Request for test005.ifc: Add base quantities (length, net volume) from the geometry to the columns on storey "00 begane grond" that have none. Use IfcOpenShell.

First a look at what the model holds.

```python
import ifcopenshell
import ifcopenshell.util.element
import ifcopenshell.util.unit

model = ifcopenshell.open("test005.ifc")
print(model.schema)
for unit_type in ("LENGTHUNIT", "AREAUNIT", "VOLUMEUNIT"):
    print(unit_type, ifcopenshell.util.unit.calculate_unit_scale(model, unit_type))
storey = next(s for s in model.by_type("IfcBuildingStorey") if s.Name == "00 begane grond")
columns = [e for e in ifcopenshell.util.element.get_decomposition(storey) if e.is_a("IfcColumn")]
for e in sorted(columns, key=lambda e: e.id()):
    print(e.id(), e.is_a(), e.Name, list(ifcopenshell.util.element.get_psets(e, qtos_only=True)), sep=" | ")
```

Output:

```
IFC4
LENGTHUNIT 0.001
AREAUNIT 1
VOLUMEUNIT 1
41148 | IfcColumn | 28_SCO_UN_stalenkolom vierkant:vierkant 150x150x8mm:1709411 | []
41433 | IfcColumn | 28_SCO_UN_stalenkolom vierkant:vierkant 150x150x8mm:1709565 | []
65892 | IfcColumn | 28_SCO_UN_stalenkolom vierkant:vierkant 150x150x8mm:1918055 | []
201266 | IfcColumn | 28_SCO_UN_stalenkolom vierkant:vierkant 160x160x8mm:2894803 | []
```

```python
import ifcopenshell
import ifcopenshell.api.pset
import ifcopenshell.geom
import ifcopenshell.util.element
import ifcopenshell.util.shape
import ifcopenshell.util.unit

model = ifcopenshell.open("test005.ifc")
unit_scale = ifcopenshell.util.unit.calculate_unit_scale(model)
volume_scale = ifcopenshell.util.unit.calculate_unit_scale(model, "VOLUMEUNIT")
settings = ifcopenshell.geom.settings()

storey = next(s for s in model.by_type("IfcBuildingStorey") if s.Name == "00 begane grond")
columns = [e for e in ifcopenshell.util.element.get_decomposition(storey) if e.is_a("IfcColumn")]

for e in sorted(columns, key=lambda e: e.id()):
    if ifcopenshell.util.element.get_psets(e, qtos_only=True, should_inherit=False):
        continue
    # Geometry comes back in metres, in the element's own axes.
    shape = ifcopenshell.geom.create_shape(settings, e)
    values = {
        "Length": ifcopenshell.util.shape.get_z(shape.geometry) / unit_scale,
        "NetVolume": ifcopenshell.util.shape.get_volume(shape.geometry) / volume_scale,
    }
    qto = ifcopenshell.api.pset.add_qto(model, product=e, name="Qto_ColumnBaseQuantities")
    ifcopenshell.api.pset.edit_qto(model, qto=qto, properties=values)
    print(e.id(), {k: round(v, 3) for k, v in values.items()})

model.write("test005_updated.ifc")
```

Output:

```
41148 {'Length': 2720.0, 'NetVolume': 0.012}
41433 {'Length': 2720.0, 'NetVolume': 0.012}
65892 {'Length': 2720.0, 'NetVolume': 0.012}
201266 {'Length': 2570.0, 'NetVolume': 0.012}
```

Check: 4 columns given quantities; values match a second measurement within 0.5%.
